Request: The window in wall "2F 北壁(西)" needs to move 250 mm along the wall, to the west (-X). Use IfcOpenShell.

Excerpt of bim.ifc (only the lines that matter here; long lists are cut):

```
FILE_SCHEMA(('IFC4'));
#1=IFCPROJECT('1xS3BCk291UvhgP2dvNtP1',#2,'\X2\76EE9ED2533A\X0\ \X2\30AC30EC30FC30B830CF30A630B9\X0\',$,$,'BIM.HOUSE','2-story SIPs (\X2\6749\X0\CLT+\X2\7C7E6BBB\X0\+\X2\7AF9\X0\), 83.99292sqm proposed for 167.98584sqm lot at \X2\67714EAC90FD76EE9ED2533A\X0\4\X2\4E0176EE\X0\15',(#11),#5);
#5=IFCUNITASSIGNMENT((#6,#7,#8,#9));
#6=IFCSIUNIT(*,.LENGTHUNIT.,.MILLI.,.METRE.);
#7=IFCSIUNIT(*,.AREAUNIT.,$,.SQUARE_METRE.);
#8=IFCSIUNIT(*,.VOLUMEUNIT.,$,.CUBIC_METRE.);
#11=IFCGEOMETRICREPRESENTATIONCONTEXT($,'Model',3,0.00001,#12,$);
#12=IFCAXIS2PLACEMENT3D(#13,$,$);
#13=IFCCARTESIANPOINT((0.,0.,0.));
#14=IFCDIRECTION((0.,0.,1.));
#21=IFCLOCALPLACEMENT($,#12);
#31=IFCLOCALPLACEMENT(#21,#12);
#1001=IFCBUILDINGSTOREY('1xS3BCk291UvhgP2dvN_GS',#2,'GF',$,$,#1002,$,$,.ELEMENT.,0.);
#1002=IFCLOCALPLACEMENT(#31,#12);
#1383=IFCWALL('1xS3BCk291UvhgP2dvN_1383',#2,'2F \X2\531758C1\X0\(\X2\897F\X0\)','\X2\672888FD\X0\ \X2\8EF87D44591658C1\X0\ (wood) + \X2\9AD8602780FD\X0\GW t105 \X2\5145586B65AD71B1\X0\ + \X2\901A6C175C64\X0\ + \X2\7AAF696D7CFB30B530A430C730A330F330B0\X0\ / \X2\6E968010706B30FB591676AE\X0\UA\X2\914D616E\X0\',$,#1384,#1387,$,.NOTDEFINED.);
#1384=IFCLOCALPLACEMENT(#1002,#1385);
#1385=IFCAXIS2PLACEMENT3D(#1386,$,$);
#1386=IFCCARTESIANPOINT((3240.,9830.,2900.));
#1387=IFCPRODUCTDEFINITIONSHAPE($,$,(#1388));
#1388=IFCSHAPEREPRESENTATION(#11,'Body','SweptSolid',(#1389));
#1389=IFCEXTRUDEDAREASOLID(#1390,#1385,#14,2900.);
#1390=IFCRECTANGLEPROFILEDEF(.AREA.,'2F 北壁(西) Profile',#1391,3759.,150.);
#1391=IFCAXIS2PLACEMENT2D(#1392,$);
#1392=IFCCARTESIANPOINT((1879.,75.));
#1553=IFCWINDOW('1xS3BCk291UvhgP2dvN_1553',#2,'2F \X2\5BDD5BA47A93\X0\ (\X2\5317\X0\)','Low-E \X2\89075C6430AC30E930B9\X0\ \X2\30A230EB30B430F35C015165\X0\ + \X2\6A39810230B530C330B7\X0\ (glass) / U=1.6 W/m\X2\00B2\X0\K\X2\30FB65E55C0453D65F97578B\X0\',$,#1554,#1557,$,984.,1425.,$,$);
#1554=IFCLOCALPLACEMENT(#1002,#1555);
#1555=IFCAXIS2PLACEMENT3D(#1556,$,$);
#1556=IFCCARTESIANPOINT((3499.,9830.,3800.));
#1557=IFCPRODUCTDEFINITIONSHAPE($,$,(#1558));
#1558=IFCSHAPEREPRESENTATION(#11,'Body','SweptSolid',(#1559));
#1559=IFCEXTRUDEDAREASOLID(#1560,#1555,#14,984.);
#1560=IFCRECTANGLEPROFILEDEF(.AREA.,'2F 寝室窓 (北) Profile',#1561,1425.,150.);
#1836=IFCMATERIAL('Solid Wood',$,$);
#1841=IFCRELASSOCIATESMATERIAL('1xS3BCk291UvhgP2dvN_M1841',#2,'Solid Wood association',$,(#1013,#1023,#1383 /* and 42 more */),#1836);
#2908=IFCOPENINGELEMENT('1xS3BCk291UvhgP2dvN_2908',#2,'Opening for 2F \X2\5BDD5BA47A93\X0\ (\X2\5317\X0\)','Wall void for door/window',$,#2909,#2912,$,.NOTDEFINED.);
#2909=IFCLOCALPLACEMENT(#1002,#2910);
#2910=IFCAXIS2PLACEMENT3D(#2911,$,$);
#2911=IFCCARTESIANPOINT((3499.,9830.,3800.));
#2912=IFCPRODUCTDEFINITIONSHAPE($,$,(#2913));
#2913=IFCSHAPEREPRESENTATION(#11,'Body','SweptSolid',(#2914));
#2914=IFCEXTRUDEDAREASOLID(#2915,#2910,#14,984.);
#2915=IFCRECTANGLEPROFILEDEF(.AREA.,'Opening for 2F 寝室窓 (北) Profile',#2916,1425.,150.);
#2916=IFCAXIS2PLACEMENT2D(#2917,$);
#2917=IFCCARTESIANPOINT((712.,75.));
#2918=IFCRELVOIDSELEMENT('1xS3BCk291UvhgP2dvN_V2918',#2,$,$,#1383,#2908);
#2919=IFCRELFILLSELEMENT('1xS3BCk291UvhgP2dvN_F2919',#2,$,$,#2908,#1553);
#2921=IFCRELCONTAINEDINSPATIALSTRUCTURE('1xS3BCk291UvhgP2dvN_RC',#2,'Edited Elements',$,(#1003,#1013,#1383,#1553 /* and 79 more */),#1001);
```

```python
import ifcopenshell
import ifcopenshell.api.geometry
import ifcopenshell.util.placement
import ifcopenshell.util.unit

model = ifcopenshell.open("bim.ifc")
unit_scale = ifcopenshell.util.unit.calculate_unit_scale(model)

window = model.by_guid("1xS3BCk291UvhgP2dvN_1553")
opening = window.FillsVoids[0].RelatingOpeningElement
wall = opening.VoidsElements[0].RelatingBuildingElement

wall_matrix = ifcopenshell.util.placement.get_local_placement(wall.ObjectPlacement)
shift = wall_matrix[:3, 0] * -0.25 / unit_scale
before = ifcopenshell.util.placement.get_local_placement(window.ObjectPlacement)[:3, 3].copy()

# The window is not placed relative to its opening, so move both.
for product in (opening, window):
    matrix = ifcopenshell.util.placement.get_local_placement(product.ObjectPlacement)
    matrix[:3, 3] += shift
    ifcopenshell.api.geometry.edit_object_placement(model, product=product, matrix=matrix, is_si=False)

after = ifcopenshell.util.placement.get_local_placement(window.ObjectPlacement)[:3, 3]
print("window moved by", (after - before).round(3) + 0.0)

model.write("bim_updated.ifc")
```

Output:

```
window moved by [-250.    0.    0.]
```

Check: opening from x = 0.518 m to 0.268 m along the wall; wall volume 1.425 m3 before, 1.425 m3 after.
